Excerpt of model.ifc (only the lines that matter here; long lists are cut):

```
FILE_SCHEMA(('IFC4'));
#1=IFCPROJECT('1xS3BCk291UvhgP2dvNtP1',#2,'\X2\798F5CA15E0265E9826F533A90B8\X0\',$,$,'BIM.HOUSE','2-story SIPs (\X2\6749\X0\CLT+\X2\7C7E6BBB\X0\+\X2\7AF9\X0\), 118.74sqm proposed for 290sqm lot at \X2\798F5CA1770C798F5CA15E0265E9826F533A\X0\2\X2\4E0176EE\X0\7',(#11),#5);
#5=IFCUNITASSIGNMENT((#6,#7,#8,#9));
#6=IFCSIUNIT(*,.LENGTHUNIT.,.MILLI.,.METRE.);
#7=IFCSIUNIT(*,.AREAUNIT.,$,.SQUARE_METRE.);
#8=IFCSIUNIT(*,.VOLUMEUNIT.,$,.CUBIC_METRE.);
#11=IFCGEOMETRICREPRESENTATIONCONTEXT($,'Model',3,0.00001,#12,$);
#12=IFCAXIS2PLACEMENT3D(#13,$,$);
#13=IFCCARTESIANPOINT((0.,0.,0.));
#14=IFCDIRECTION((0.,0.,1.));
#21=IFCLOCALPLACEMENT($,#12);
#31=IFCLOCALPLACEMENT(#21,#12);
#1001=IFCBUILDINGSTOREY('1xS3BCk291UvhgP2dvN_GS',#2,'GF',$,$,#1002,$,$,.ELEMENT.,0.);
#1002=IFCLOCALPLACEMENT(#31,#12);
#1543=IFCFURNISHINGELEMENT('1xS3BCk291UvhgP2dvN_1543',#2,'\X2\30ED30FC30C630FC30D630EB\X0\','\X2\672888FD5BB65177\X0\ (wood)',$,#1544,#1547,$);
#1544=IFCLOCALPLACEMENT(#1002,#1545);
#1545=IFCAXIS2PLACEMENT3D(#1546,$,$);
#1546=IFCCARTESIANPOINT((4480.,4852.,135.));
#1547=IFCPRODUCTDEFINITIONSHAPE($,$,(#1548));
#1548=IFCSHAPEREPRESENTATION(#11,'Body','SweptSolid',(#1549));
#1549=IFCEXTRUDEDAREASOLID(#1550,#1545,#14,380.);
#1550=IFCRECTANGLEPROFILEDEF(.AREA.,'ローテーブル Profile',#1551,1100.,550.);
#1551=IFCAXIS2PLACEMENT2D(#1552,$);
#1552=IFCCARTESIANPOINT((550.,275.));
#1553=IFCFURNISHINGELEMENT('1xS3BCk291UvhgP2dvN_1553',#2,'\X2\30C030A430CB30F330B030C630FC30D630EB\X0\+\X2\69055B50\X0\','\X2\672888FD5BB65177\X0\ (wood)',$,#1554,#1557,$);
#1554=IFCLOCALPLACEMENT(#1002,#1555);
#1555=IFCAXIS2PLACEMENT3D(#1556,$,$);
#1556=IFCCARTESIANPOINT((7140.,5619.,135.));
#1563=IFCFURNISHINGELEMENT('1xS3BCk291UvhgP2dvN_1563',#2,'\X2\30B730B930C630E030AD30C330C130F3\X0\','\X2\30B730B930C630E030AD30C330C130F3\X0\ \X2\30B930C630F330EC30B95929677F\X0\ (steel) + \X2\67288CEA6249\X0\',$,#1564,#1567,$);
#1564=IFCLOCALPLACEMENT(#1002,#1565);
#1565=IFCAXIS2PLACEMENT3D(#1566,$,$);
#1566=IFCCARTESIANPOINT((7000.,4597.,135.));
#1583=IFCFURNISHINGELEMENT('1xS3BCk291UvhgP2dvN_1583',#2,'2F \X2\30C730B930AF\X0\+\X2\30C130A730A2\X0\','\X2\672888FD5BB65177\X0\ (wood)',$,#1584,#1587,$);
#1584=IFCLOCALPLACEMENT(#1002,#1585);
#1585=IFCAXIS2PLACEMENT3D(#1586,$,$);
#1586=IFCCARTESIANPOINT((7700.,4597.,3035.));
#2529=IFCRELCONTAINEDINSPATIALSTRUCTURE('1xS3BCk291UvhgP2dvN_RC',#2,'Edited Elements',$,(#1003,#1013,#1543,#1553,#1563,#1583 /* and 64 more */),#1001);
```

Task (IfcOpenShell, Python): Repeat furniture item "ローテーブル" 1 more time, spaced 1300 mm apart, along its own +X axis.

```python
import ifcopenshell
import ifcopenshell.api.geometry
import ifcopenshell.api.root
import ifcopenshell.util.element
import ifcopenshell.util.placement
import ifcopenshell.util.unit

model = ifcopenshell.open("model.ifc")
unit_scale = ifcopenshell.util.unit.calculate_unit_scale(model)


def reuse_history(source, copy):
    """copy_class also copies each property set's owner history, people and application; keep the originals."""
    for rel in copy.IsDefinedBy:
        if rel.is_a("IfcRelDefinesByProperties") and (history := rel.RelatingPropertyDefinition.OwnerHistory):
            rel.RelatingPropertyDefinition.OwnerHistory = source.OwnerHistory
            ifcopenshell.util.element.remove_deep2(model, history)


source = model.by_guid("1xS3BCk291UvhgP2dvN_1543")
base = ifcopenshell.util.placement.get_local_placement(source.ObjectPlacement)
step = base[:3, 0] * 1.3 / unit_scale

for i in range(1, 2):
    copy = ifcopenshell.api.root.copy_class(model, product=source)
    copy.Representation = ifcopenshell.util.element.copy_deep(
        model, source.Representation, exclude=["IfcGeometricRepresentationContext", "IfcRepresentationMap"]
    )
    reuse_history(source, copy)
    matrix = base.copy()
    matrix[:3, 3] += i * step
    print("added at", matrix[:3, 3].round(3) + 0.0)
    ifcopenshell.api.geometry.edit_object_placement(model, product=copy, matrix=matrix, is_si=False)

model.write("model-out.ifc")
```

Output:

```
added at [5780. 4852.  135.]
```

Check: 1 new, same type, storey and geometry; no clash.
